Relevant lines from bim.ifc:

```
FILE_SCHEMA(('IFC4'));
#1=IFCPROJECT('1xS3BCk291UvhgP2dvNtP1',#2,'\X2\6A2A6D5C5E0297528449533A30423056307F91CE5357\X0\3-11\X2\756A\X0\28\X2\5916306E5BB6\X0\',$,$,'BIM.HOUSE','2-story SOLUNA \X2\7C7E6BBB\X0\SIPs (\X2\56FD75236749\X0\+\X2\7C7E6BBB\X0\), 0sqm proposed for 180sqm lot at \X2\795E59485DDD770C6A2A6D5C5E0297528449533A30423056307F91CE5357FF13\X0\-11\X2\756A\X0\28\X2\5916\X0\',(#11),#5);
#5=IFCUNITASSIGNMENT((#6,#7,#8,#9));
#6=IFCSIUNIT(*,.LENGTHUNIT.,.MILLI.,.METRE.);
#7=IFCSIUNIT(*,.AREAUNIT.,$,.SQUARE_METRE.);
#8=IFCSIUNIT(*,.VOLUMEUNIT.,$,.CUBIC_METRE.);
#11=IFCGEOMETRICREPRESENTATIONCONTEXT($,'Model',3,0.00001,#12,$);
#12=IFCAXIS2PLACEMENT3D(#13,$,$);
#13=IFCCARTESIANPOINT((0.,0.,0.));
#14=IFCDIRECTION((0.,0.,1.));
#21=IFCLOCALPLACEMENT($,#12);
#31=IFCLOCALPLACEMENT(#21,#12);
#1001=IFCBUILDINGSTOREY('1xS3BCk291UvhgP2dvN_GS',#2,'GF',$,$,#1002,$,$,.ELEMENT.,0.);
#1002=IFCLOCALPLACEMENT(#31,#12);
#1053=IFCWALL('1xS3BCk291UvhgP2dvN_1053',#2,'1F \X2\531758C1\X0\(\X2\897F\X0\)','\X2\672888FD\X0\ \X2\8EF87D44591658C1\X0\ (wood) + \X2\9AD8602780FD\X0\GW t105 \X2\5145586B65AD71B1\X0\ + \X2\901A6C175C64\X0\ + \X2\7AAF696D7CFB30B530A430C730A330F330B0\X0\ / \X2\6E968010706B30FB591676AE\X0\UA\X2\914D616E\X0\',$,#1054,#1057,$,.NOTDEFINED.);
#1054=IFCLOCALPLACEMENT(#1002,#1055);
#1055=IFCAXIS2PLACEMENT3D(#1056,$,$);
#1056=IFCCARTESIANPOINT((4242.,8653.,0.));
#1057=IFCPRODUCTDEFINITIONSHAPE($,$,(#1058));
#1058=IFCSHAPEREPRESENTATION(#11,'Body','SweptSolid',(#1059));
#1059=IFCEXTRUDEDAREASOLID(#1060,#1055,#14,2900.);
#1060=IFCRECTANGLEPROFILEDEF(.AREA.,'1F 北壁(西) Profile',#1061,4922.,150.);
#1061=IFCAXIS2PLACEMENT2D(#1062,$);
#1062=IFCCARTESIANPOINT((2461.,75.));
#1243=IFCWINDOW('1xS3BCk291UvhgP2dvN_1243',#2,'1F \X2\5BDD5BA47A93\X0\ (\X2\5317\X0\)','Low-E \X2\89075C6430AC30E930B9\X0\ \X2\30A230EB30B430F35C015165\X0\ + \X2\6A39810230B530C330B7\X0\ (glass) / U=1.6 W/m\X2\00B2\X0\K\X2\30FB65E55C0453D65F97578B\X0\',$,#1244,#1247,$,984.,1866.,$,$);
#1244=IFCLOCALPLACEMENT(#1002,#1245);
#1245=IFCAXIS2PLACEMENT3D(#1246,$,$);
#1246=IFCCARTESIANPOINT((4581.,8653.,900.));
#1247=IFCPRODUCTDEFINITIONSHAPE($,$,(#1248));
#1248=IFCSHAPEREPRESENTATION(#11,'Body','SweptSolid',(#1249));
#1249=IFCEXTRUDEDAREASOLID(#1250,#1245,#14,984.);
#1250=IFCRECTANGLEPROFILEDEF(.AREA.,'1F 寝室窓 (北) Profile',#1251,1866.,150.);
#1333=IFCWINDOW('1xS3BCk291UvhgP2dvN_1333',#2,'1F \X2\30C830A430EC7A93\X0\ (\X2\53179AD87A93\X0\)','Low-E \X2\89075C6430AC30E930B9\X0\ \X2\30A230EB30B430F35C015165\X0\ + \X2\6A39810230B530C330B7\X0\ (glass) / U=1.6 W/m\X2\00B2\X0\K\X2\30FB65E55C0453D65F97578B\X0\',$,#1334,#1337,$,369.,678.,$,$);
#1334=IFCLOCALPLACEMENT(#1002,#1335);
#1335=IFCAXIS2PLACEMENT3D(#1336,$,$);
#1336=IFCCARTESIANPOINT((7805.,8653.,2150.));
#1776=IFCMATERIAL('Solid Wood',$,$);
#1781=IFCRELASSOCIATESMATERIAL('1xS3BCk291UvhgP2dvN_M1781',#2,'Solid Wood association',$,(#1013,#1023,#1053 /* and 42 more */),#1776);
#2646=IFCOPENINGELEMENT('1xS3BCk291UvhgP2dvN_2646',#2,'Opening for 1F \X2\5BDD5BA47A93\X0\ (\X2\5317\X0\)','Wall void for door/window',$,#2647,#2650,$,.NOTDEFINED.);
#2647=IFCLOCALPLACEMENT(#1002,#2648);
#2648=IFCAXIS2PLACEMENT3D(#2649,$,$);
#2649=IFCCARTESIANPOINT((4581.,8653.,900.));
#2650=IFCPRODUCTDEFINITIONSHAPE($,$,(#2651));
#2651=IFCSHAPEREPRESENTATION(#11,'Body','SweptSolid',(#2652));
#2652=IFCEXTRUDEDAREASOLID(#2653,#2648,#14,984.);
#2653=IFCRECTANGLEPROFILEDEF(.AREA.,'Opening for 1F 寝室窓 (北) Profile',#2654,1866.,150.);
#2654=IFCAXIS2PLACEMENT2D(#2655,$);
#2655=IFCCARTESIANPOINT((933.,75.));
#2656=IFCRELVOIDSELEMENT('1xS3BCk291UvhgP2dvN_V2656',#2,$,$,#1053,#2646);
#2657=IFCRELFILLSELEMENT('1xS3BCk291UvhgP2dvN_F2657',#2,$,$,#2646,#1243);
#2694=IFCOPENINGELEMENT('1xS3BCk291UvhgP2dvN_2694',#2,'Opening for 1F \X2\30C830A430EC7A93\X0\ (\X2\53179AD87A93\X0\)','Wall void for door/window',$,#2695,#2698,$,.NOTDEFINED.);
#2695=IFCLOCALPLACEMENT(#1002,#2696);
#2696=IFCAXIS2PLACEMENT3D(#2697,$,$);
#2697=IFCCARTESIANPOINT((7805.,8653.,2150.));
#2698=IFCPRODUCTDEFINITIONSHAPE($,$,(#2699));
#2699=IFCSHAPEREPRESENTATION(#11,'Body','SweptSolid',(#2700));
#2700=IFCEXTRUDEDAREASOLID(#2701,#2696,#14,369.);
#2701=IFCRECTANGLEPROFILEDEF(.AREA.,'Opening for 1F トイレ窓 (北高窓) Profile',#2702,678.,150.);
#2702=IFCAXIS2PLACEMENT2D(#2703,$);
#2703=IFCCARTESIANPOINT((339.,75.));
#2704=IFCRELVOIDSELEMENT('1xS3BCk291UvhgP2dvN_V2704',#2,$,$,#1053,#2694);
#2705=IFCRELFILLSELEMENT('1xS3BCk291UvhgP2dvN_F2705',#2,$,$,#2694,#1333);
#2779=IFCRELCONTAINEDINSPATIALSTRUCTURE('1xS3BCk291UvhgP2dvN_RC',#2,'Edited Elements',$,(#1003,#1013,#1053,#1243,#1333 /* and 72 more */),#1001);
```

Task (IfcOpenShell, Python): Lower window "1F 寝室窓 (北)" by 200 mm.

```python
import numpy as np
import ifcopenshell
import ifcopenshell.api.geometry
import ifcopenshell.util.placement
import ifcopenshell.util.unit

model = ifcopenshell.open("bim.ifc")
unit_scale = ifcopenshell.util.unit.calculate_unit_scale(model)

window = model.by_id(1243)
opening = window.FillsVoids[0].RelatingOpeningElement
dz = -0.2 / unit_scale

shift = np.array([0.0, 0.0, dz])
# The window is not placed relative to its opening, so move both.
for product in (opening, window):
    matrix = ifcopenshell.util.placement.get_local_placement(product.ObjectPlacement)
    matrix[:3, 3] += shift
    ifcopenshell.api.geometry.edit_object_placement(model, product=product, matrix=matrix, is_si=False)

print(f"moved by {dz * unit_scale:+.3f} m")

model.write("bim-out.ifc")
```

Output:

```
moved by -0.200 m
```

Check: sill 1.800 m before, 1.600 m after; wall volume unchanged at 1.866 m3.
